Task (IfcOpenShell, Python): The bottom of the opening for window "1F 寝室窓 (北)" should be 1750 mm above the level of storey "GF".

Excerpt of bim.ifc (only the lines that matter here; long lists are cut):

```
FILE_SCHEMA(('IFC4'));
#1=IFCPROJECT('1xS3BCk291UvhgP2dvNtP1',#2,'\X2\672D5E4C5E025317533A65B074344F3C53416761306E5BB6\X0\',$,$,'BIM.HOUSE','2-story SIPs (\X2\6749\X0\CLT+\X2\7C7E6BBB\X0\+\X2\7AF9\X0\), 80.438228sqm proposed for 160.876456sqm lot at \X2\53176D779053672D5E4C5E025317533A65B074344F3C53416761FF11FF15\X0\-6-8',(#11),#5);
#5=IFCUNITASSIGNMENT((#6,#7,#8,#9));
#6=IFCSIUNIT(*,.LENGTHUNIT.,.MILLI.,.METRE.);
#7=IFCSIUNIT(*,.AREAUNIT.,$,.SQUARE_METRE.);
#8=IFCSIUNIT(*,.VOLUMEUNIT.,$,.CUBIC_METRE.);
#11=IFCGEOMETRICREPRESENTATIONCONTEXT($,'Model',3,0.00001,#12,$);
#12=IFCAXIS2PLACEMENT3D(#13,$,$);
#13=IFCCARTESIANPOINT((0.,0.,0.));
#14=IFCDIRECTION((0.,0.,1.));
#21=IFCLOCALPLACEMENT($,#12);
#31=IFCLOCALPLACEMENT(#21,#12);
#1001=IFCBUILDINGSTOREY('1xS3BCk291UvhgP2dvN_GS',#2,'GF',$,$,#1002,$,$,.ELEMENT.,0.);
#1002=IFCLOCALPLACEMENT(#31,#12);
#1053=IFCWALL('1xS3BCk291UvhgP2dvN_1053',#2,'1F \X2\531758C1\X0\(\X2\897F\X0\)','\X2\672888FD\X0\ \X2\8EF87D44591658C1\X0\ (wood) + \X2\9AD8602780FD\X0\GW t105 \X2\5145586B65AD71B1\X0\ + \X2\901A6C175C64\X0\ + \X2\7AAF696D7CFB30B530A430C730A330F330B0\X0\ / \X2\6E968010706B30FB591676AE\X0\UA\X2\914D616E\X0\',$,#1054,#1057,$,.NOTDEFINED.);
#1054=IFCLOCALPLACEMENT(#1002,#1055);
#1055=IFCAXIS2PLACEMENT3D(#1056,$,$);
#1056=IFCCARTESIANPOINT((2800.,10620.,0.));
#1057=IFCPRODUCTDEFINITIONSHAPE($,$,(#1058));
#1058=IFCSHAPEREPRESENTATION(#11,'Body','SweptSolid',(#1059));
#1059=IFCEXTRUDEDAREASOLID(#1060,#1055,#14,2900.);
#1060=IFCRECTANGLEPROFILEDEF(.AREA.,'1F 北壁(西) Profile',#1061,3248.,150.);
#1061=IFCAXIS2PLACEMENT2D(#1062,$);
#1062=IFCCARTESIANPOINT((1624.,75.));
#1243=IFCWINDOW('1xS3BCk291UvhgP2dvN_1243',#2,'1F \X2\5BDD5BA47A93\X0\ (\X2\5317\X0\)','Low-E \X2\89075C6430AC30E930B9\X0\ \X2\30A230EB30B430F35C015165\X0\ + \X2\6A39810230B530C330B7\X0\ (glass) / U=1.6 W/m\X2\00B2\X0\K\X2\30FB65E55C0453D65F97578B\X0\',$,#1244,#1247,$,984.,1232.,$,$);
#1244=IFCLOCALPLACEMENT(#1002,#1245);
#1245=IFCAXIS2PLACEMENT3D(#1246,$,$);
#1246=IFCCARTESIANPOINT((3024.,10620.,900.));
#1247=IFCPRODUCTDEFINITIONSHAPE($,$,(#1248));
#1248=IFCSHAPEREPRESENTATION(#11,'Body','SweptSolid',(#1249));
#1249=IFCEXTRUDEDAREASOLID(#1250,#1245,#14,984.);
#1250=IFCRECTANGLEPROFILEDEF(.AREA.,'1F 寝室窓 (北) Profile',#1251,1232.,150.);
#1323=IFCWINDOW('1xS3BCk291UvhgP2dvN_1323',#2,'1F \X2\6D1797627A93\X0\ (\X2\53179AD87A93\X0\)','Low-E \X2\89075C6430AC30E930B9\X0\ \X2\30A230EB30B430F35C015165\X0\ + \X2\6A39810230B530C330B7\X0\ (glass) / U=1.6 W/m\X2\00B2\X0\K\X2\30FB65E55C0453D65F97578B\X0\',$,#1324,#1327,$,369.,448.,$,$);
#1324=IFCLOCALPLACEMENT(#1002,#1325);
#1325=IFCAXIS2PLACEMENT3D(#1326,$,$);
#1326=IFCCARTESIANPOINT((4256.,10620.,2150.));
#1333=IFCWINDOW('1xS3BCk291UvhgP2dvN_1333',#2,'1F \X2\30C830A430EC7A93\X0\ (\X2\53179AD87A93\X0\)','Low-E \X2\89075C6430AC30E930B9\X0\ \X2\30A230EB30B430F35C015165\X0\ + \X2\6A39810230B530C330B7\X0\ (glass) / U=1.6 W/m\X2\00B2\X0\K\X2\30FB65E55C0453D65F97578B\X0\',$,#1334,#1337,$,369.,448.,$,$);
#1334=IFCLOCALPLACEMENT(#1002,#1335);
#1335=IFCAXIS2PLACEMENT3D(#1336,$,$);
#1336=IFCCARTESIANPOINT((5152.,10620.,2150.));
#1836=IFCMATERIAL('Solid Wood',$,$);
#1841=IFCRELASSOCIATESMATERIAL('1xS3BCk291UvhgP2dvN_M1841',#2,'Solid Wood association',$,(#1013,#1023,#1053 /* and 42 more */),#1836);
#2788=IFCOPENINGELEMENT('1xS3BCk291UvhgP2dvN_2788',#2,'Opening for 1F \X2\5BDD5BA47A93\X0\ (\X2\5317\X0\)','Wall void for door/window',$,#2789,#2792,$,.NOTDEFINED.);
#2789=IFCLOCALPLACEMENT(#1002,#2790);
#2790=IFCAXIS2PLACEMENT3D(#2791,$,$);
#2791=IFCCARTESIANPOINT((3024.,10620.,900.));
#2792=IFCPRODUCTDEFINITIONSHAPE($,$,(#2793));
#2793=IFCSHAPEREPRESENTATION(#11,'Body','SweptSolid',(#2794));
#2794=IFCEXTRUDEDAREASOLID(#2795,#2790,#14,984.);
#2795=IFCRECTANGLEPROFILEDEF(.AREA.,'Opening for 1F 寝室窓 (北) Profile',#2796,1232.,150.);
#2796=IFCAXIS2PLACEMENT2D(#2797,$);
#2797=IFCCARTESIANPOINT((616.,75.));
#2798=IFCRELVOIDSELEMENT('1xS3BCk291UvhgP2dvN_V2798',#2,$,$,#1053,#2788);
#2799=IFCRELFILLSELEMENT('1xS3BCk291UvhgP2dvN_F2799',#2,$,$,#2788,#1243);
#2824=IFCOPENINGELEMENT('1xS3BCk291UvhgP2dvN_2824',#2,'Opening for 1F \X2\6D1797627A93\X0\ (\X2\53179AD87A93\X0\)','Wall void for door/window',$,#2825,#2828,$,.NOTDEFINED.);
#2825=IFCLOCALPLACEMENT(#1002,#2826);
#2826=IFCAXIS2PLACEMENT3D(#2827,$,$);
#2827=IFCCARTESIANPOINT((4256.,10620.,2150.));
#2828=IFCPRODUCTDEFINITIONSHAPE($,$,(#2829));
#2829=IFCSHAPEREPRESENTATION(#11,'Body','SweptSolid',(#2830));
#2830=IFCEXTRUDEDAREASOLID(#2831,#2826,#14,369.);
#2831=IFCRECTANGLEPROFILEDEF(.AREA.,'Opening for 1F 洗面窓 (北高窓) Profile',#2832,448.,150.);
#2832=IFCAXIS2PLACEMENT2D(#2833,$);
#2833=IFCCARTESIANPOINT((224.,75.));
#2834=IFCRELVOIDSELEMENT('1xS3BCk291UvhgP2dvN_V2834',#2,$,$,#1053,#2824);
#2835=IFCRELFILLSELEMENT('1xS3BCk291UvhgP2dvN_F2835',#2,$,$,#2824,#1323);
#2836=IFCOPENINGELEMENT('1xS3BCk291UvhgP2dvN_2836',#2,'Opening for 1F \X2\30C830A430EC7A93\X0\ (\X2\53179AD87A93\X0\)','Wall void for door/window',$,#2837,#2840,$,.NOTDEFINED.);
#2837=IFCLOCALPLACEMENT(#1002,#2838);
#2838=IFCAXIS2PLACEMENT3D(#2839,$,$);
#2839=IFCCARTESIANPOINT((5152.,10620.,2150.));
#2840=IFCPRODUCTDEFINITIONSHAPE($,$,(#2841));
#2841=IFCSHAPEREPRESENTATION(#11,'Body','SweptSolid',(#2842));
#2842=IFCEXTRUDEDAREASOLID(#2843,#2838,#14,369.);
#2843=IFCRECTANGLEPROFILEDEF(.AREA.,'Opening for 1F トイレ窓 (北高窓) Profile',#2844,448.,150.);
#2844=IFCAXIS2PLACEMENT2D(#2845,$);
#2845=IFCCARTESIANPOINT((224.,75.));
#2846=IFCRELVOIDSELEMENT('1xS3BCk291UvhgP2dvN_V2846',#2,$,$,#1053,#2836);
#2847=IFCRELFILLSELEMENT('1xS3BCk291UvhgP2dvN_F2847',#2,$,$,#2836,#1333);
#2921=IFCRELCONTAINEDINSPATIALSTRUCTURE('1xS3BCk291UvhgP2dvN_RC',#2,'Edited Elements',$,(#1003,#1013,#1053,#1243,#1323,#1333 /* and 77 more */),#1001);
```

```python
import numpy as np
import ifcopenshell
import ifcopenshell.api.geometry
import ifcopenshell.geom
import ifcopenshell.util.element
import ifcopenshell.util.placement
import ifcopenshell.util.shape
import ifcopenshell.util.unit

model = ifcopenshell.open("bim.ifc")
unit_scale = ifcopenshell.util.unit.calculate_unit_scale(model)

window = model.by_guid("1xS3BCk291UvhgP2dvN_1243")
opening = window.FillsVoids[0].RelatingOpeningElement
storey = ifcopenshell.util.element.get_container(window, ifc_class="IfcBuildingStorey")
level = ifcopenshell.util.placement.get_local_placement(storey.ObjectPlacement)[2, 3]

# The opening's origin need not be at the sill, so measure its lowest point.
shape = ifcopenshell.geom.create_shape(ifcopenshell.geom.settings(), opening)
bottom = ifcopenshell.util.shape.get_shape_bottom_elevation(shape, shape.geometry) / unit_scale
dz = level + 1750.0 - bottom

shift = np.array([0.0, 0.0, dz])
# The window is not placed relative to its opening, so move both.
for product in (opening, window):
    matrix = ifcopenshell.util.placement.get_local_placement(product.ObjectPlacement)
    matrix[:3, 3] += shift
    ifcopenshell.api.geometry.edit_object_placement(model, product=product, matrix=matrix, is_si=False)

print(f"moved by {dz * unit_scale:+.3f} m")

model.write("bim_updated.ifc")
```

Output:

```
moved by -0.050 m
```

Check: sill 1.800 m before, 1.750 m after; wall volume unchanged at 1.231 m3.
